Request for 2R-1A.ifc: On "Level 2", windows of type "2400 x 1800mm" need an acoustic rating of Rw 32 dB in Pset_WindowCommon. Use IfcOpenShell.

First a look at what the model holds.

```python
import ifcopenshell
import ifcopenshell.util.element

model = ifcopenshell.open("2R-1A.ifc")
print(model.schema)
storey = next(s for s in model.by_type("IfcBuildingStorey") if s.Name == "Level 2")
windows = [e for e in ifcopenshell.util.element.get_decomposition(storey) if e.is_a("IfcWindow")]
seen = {}
for e in windows:
    element_type = ifcopenshell.util.element.get_type(e)
    key = (element_type.Name if element_type != e and element_type else None, ifcopenshell.util.element.get_pset(e, "Pset_WindowCommon", "AcousticRating"))
    seen[key] = seen.get(key, 0) + 1
for (name, value), count in sorted(seen.items(), key=str):
    print(count, "x", name, "|", value)
```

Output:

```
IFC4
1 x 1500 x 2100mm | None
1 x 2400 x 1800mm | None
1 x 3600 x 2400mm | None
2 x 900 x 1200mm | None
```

```python
import ifcopenshell
import ifcopenshell.api.pset
import ifcopenshell.util.element

model = ifcopenshell.open("2R-1A.ifc")

storey = next(s for s in model.by_type("IfcBuildingStorey") if s.Name == "Level 2")
windows = [e for e in ifcopenshell.util.element.get_decomposition(storey) if e.is_a("IfcWindow")]

count = 0
for e in windows:
    element_type = ifcopenshell.util.element.get_type(e)
    if element_type in (None, e) or element_type.Name != "2400 x 1800mm":
        continue
    # add_pset returns the element's existing set when there is one.
    pset = ifcopenshell.api.pset.add_pset(model, product=e, name="Pset_WindowCommon")
    ifcopenshell.api.pset.edit_pset(model, pset=pset, properties={"AcousticRating": "Rw 32 dB"})
    count += 1

print(count, "windows updated")

model.write("2R-1A_edited.ifc")
```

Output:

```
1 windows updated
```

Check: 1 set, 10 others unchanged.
